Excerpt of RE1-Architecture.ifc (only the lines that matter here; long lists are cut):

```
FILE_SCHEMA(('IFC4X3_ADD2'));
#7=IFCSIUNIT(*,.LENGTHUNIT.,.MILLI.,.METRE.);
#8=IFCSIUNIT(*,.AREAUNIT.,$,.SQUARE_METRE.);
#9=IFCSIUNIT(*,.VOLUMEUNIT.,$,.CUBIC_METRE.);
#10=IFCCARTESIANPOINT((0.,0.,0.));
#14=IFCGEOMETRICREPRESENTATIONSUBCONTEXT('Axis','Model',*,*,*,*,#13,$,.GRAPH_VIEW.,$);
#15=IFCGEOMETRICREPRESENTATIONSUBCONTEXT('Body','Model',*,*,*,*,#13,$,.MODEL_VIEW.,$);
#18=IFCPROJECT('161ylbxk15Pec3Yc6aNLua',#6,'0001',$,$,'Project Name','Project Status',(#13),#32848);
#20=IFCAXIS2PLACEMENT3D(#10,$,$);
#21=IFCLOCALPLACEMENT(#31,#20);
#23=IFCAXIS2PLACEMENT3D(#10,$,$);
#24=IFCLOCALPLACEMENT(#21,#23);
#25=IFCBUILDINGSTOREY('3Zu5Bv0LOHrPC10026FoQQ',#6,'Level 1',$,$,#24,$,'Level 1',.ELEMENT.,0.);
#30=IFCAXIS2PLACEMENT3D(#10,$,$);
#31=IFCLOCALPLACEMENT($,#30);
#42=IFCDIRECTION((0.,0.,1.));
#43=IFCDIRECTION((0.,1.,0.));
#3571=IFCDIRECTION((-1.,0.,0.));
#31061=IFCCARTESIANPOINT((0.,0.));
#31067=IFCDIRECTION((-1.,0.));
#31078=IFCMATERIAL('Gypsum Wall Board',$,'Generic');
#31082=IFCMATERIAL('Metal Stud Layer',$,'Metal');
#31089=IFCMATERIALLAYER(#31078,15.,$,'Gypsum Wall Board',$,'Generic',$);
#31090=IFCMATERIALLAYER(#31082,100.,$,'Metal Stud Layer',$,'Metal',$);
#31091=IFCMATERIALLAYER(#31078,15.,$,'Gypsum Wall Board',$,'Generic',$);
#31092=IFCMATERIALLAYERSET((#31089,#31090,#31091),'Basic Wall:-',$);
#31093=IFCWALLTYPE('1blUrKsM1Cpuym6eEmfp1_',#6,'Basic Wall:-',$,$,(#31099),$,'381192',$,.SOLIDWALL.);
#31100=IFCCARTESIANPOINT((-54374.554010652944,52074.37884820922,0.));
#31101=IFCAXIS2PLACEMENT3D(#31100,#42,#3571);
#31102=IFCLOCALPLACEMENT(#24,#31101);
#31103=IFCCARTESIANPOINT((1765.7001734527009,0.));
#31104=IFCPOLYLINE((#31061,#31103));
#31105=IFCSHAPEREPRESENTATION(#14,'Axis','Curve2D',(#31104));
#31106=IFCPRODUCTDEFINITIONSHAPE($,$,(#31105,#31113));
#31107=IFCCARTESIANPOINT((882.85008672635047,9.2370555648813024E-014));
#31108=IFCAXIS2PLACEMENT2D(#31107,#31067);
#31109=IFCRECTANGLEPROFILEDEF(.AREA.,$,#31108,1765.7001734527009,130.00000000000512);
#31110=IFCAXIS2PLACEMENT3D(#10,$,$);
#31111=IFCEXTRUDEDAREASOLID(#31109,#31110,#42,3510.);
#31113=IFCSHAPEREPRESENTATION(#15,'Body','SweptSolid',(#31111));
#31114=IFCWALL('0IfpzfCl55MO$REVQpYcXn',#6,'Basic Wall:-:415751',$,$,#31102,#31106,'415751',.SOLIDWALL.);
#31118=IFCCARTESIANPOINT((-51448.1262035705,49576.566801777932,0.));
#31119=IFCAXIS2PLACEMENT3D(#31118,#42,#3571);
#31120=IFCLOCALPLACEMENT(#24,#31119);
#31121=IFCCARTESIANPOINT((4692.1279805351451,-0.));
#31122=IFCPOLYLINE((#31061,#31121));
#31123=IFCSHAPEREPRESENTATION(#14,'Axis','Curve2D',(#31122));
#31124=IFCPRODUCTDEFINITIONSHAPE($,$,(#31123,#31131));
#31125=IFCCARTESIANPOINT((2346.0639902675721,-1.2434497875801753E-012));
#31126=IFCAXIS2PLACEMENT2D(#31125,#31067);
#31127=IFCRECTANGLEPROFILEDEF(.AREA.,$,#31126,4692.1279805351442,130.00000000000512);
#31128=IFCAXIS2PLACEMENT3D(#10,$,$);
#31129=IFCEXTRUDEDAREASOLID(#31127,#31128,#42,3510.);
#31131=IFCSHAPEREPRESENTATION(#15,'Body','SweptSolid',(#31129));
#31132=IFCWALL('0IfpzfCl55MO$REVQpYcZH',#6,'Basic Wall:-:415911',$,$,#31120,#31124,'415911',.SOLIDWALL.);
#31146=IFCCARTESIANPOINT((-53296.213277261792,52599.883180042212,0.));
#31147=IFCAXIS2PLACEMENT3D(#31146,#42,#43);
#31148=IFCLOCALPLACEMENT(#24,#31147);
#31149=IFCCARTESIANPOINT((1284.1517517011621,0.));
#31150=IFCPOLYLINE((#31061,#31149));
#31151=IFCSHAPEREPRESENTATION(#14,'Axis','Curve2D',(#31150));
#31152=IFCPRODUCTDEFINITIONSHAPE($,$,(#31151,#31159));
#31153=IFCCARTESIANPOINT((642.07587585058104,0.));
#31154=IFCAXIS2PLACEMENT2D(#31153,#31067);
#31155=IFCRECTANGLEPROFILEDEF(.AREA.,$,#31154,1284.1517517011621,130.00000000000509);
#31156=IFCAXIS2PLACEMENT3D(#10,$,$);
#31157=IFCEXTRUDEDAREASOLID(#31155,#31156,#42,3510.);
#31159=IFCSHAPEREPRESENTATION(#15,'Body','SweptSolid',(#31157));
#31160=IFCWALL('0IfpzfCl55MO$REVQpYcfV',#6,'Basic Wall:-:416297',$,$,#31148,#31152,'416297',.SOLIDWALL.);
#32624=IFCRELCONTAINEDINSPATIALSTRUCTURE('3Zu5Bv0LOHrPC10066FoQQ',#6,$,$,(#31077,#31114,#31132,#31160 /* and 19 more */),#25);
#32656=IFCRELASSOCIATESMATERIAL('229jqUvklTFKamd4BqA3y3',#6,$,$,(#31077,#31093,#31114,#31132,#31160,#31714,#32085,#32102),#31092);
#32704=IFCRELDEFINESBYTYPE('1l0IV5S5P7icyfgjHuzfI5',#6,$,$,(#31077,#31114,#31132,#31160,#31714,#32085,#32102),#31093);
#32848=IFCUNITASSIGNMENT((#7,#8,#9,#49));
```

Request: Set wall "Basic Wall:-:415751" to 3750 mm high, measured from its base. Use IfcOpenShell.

```python
import ifcopenshell
import ifcopenshell.geom
import ifcopenshell.util.representation
import ifcopenshell.util.shape

model = ifcopenshell.open("RE1-Architecture.ifc")
settings = ifcopenshell.geom.settings()


def volume(element):
    """Net volume in cubic metres, openings subtracted."""
    shape = ifcopenshell.geom.create_shape(settings, element)
    return ifcopenshell.util.shape.get_volume(shape.geometry)


wall = model.by_guid("0IfpzfCl55MO$REVQpYcXn")
before = volume(wall)

body = ifcopenshell.util.representation.get_representation(wall, "Model", "Body")
solid = body.Items[0]
old_height = solid.Depth
solid.Depth = 3750.0
after = volume(wall)

print(f"height {old_height:g} -> {solid.Depth:g}, volume {before:.3f} -> {after:.3f} m3")

model.write("RE1-Architecture_updated.ifc")
```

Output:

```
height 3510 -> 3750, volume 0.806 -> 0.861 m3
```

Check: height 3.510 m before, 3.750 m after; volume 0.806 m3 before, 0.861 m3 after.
